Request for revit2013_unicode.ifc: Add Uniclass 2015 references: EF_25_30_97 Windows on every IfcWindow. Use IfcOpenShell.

First a look at what the model holds.

```python
import ifcopenshell

model = ifcopenshell.open("revit2013_unicode.ifc")
print(model.schema)
print("classifications:", [c.Name for c in model.by_type("IfcClassification")])
for ifc_class in ("IfcDoor", "IfcRoof", "IfcStair", "IfcWall", "IfcWindow"):
    print(ifc_class, len(model.by_type(ifc_class)))
```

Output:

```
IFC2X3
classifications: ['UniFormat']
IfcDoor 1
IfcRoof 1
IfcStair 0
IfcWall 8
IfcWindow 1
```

```python
import ifcopenshell
import ifcopenshell.api.classification

model = ifcopenshell.open("revit2013_unicode.ifc")

# IFC2X3 requires Source and Edition and has no link from the project to the system.
system = model.create_entity("IfcClassification", Source="NBS", Edition="2015", Name="Uniclass 2015")

codes = {
    "IfcWindow": ("EF_25_30_97", "Windows"),
}
for ifc_class, (code, name) in codes.items():
    products = model.by_type(ifc_class)
    ifcopenshell.api.classification.add_reference(
        model, products=products, classification=system, identification=code, name=name
    )
    print(code, len(products))

model.write("revit2013_unicode_updated.ifc")
```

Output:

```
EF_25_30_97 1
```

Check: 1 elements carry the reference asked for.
